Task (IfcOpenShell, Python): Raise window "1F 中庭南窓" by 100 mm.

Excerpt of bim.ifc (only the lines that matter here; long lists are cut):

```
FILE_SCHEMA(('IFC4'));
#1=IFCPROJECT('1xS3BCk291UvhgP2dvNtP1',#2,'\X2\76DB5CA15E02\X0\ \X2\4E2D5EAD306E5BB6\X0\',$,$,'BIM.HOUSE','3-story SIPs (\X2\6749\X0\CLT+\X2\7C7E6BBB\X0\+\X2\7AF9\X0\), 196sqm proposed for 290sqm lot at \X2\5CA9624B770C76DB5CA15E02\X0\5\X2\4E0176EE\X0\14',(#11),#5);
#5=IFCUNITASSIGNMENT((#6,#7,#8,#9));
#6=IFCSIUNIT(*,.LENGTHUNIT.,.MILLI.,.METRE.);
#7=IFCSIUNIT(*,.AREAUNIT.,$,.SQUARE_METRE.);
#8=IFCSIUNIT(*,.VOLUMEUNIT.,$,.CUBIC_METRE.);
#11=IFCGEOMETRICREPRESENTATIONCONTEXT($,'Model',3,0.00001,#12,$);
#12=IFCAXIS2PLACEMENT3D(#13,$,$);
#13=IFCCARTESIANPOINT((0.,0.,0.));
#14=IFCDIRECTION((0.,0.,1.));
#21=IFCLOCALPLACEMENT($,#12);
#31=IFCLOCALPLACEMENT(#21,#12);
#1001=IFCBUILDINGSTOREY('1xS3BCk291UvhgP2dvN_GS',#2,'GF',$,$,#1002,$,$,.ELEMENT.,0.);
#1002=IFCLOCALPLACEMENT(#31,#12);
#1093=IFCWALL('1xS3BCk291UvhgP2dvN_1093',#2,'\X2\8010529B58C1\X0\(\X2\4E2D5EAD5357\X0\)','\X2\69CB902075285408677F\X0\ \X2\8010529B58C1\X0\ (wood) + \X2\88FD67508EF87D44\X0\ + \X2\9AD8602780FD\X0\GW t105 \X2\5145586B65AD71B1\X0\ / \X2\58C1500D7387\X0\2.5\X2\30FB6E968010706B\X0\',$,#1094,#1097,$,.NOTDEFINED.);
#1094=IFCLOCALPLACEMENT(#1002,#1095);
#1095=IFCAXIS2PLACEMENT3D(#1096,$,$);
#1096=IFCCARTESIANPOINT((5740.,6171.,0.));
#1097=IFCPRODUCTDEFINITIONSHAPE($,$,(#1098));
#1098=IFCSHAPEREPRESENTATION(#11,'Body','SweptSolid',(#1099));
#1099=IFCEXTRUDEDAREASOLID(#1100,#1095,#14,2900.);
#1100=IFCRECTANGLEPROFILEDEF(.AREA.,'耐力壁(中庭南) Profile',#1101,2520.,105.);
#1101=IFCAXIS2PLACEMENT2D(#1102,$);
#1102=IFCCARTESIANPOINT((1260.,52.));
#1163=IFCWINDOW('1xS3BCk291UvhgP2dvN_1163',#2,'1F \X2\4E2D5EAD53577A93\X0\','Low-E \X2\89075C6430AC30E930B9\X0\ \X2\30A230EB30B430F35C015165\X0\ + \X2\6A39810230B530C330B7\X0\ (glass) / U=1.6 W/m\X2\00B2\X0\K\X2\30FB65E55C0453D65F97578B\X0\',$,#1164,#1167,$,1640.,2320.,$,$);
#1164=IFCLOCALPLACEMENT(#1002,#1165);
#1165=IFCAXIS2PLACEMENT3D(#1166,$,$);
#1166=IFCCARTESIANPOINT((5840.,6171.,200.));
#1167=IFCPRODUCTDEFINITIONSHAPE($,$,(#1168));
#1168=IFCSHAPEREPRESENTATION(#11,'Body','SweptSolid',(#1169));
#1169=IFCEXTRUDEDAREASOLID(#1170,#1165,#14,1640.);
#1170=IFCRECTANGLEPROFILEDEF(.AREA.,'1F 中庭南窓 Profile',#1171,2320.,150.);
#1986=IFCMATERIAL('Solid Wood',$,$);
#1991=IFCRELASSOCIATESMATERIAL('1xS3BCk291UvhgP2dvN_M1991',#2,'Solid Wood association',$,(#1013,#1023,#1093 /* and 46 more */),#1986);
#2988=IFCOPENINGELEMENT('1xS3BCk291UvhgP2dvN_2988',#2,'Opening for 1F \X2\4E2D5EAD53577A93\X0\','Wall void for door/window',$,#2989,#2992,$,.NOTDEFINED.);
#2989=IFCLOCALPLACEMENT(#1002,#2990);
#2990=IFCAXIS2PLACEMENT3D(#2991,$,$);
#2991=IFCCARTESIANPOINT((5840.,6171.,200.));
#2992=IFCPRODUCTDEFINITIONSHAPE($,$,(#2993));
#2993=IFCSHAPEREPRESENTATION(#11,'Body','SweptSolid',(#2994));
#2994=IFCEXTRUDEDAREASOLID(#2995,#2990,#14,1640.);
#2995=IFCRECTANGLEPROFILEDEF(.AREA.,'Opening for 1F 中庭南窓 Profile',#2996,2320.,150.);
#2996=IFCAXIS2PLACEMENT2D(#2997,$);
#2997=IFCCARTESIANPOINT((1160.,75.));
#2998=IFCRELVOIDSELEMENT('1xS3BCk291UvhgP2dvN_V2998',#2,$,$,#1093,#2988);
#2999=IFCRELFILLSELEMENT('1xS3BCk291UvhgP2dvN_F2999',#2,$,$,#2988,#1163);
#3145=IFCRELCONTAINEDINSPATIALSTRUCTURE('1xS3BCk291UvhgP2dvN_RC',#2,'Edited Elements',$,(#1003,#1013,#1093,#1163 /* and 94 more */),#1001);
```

```python
import numpy as np
import ifcopenshell
import ifcopenshell.api.geometry
import ifcopenshell.util.placement
import ifcopenshell.util.unit

model = ifcopenshell.open("bim.ifc")
unit_scale = ifcopenshell.util.unit.calculate_unit_scale(model)

window = model.by_guid("1xS3BCk291UvhgP2dvN_1163")
opening = window.FillsVoids[0].RelatingOpeningElement
dz = 0.1 / unit_scale

shift = np.array([0.0, 0.0, dz])
# The window is not placed relative to its opening, so move both.
for product in (opening, window):
    matrix = ifcopenshell.util.placement.get_local_placement(product.ObjectPlacement)
    matrix[:3, 3] += shift
    ifcopenshell.api.geometry.edit_object_placement(model, product=product, matrix=matrix, is_si=False)

print(f"moved by {dz * unit_scale:+.3f} m")

model.write("bim_v2.ifc")
```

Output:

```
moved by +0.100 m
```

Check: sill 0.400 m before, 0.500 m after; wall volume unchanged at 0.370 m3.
